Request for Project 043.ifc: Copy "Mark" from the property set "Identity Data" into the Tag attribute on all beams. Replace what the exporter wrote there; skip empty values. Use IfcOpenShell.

First a look at what the model holds.

```python
import ifcopenshell
import ifcopenshell.util.element

model = ifcopenshell.open("Project 043.ifc")
print(model.schema)
beams = model.by_type("IfcBeam")
print(len(beams), "beams")
for e in beams[:8]:
    source = ifcopenshell.util.element.get_pset(e, "Identity Data", "Mark")
    target = e.Tag
    print(e.id(), repr(source), repr(target), sep=" | ")
```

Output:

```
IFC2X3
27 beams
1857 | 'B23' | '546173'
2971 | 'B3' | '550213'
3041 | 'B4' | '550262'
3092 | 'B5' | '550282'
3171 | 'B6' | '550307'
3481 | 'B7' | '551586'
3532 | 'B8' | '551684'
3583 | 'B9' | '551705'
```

```python
import ifcopenshell
import ifcopenshell.util.element

model = ifcopenshell.open("Project 043.ifc")

count = 0
for e in model.by_type("IfcBeam"):
    value = ifcopenshell.util.element.get_pset(e, "Identity Data", "Mark")
    current = e.Tag
    if not value or not value.strip() or current == value:
        continue
    e.Tag = value
    count += 1

print(count, "beams updated")

model.write("Project 043_rev.ifc")
```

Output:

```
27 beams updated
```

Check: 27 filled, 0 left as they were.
